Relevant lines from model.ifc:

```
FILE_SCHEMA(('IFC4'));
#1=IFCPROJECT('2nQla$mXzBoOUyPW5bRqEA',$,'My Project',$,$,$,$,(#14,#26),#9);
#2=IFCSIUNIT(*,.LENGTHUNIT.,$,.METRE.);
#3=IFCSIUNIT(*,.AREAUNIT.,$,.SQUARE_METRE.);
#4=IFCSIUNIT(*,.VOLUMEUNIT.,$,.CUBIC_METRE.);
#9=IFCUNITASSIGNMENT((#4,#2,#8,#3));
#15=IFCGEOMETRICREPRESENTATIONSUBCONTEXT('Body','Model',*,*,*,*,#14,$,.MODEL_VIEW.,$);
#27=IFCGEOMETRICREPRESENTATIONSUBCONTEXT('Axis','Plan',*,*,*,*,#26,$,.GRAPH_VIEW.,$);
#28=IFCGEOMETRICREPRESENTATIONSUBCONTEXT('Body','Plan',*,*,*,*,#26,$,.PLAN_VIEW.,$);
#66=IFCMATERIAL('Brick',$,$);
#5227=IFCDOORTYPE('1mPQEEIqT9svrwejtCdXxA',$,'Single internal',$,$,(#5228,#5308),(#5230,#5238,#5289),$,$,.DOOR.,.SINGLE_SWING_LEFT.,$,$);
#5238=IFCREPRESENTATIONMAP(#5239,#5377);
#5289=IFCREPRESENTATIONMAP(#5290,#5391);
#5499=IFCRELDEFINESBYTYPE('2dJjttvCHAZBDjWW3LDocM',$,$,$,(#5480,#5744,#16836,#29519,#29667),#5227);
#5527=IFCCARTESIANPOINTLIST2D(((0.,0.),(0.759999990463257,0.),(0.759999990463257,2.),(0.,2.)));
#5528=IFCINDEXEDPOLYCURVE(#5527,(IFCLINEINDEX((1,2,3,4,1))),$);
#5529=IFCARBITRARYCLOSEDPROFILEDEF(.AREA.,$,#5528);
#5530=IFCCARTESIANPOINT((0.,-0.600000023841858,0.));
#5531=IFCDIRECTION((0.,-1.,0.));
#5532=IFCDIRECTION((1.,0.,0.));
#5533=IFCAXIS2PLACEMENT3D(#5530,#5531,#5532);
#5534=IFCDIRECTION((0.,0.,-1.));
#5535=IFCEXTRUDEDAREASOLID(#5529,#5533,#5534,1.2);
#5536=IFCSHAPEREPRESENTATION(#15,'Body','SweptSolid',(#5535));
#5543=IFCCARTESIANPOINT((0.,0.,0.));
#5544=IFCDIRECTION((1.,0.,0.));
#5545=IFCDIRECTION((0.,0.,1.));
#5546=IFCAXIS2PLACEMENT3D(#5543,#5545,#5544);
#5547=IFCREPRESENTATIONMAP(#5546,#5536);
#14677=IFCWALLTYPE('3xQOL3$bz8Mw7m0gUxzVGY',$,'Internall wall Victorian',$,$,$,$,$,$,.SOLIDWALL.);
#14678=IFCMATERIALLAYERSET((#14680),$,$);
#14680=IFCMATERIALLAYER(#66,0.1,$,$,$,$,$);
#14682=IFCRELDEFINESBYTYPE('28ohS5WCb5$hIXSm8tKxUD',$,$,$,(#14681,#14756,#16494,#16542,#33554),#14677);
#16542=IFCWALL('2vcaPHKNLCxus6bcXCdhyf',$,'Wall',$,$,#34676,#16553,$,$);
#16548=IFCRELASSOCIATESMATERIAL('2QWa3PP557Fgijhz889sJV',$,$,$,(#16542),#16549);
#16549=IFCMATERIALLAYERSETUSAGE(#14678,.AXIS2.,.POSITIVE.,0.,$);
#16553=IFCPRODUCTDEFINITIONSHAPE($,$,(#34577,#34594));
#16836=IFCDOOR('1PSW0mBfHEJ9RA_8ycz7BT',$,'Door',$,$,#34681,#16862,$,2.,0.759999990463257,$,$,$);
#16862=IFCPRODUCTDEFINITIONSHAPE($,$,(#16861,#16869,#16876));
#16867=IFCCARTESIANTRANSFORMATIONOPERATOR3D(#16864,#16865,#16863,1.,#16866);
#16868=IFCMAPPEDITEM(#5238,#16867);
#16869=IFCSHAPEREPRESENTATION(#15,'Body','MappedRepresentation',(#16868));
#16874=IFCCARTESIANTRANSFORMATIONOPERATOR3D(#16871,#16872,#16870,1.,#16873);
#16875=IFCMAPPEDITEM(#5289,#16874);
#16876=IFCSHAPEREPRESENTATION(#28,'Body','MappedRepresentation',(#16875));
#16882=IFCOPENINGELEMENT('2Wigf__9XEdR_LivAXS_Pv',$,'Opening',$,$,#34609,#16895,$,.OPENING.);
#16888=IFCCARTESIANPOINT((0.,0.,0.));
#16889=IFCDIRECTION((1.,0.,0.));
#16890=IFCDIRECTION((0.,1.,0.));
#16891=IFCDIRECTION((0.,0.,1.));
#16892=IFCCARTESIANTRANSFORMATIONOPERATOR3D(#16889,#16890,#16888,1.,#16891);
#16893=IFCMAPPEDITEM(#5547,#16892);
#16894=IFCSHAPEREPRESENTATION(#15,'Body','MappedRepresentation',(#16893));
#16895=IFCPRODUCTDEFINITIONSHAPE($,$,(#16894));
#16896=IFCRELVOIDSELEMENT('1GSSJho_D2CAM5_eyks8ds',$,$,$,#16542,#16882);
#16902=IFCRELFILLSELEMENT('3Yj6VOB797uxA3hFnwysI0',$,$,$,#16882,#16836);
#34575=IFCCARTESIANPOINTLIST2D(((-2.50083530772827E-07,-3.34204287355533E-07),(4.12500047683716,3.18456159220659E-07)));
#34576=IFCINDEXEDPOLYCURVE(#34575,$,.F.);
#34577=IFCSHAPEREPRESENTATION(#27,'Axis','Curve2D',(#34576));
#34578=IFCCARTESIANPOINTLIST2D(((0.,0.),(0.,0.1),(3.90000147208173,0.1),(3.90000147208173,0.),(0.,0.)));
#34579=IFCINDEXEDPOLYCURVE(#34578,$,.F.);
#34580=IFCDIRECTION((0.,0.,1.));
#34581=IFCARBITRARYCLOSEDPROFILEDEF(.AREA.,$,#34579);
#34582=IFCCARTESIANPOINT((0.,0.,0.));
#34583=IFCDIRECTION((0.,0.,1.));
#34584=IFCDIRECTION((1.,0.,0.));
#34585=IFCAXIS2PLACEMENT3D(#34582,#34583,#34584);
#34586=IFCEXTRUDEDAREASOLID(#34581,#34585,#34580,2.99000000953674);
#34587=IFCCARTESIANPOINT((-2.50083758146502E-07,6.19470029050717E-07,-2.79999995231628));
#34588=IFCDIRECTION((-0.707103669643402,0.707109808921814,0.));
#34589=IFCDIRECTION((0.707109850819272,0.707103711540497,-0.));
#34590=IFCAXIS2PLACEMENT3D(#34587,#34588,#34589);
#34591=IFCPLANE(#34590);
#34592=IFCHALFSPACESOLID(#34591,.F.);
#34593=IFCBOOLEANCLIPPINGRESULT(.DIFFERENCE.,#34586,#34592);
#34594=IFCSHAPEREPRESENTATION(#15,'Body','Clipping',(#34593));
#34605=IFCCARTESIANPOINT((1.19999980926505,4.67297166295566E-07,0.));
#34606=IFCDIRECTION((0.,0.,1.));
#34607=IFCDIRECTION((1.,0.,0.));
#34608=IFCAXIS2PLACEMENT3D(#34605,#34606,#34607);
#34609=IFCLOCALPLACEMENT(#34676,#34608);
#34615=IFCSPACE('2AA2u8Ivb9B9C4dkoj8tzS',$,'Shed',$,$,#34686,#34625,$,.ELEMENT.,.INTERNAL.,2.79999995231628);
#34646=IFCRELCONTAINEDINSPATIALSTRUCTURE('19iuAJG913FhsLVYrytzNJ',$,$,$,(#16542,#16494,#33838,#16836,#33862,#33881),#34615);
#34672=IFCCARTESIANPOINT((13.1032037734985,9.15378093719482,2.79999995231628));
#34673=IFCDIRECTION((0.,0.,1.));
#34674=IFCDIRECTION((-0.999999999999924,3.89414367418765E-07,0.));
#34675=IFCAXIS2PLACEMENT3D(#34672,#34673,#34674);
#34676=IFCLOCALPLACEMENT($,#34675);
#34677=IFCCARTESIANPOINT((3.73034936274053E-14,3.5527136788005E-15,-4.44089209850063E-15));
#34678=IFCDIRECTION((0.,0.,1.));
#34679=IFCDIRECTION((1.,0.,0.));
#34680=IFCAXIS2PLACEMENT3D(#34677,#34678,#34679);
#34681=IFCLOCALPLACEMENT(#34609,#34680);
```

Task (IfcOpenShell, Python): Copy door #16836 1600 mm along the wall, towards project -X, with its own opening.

```python
import ifcopenshell
import ifcopenshell.api.feature
import ifcopenshell.api.geometry
import ifcopenshell.api.root
import ifcopenshell.geom
import ifcopenshell.util.element
import ifcopenshell.util.placement
import ifcopenshell.util.shape
import ifcopenshell.util.unit

model = ifcopenshell.open("model.ifc")
unit_scale = ifcopenshell.util.unit.calculate_unit_scale(model)
settings = ifcopenshell.geom.settings()


def volume(element):
    """Net volume in cubic metres, openings subtracted."""
    shape = ifcopenshell.geom.create_shape(settings, element)
    return ifcopenshell.util.shape.get_volume(shape.geometry)


door = model.by_guid("1PSW0mBfHEJ9RA_8ycz7BT")
opening = door.FillsVoids[0].RelatingOpeningElement
wall = opening.VoidsElements[0].RelatingBuildingElement
before = volume(wall)
shift = ifcopenshell.util.placement.get_local_placement(wall.ObjectPlacement)[:3, 0] * 1.6 / unit_scale

# copy_class copies the void relationship, type, container and properties, but no geometry.
new_opening = ifcopenshell.api.root.copy_class(model, product=opening)
new_opening.Representation = ifcopenshell.util.element.copy_deep(
    model, opening.Representation, exclude=["IfcGeometricRepresentationContext", "IfcRepresentationMap"]
)
new_door = ifcopenshell.api.root.copy_class(model, product=door)
new_door.Representation = ifcopenshell.util.element.copy_deep(
    model, door.Representation, exclude=["IfcGeometricRepresentationContext", "IfcRepresentationMap"]
)
ifcopenshell.api.feature.add_filling(model, opening=new_opening, element=new_door)

for old, new in ((opening, new_opening), (door, new_door)):
    matrix = ifcopenshell.util.placement.get_local_placement(old.ObjectPlacement)
    matrix[:3, 3] += shift
    ifcopenshell.api.geometry.edit_object_placement(model, product=new, matrix=matrix, is_si=False)

after = volume(wall)

print(f"wall volume {before:.3f} -> {after:.3f} m3")

model.write("model_rev.ifc")
```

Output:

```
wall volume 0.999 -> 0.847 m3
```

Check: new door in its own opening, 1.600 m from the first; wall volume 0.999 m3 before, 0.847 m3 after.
